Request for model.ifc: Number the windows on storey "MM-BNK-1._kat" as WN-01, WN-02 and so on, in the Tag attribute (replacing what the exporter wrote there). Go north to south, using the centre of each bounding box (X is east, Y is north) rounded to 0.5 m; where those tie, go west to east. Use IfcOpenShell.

First a look at what the model holds.

```python
import ifcopenshell
import ifcopenshell.util.element
import ifcopenshell.util.placement

model = ifcopenshell.open("model.ifc")
print(model.schema)
storey = next(s for s in model.by_type("IfcBuildingStorey") if s.Name == "MM-BNK-1._kat")
windows = [e for e in ifcopenshell.util.element.get_decomposition(storey) if e.is_a("IfcWindow")]
for e in sorted(windows, key=lambda e: e.id()):
    origin = ifcopenshell.util.placement.get_local_placement(e.ObjectPlacement)[:3, 3]
    print(e.id(), e.Tag, e.Name, origin.round(2) + 0.0, sep=" | ")
```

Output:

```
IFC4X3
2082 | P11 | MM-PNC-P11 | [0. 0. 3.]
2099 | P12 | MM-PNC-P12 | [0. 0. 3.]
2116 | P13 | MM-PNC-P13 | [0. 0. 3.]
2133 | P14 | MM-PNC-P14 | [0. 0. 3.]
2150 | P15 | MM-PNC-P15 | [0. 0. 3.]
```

```python
import ifcopenshell
import ifcopenshell.geom
import ifcopenshell.util.element
import ifcopenshell.util.shape

model = ifcopenshell.open("model.ifc")
settings = ifcopenshell.geom.settings()
settings.set("use-world-coords", True)


def centre(element):
    shape = ifcopenshell.geom.create_shape(settings, element)
    return ifcopenshell.util.shape.get_bbox_centroid(shape.geometry)


storey = next(s for s in model.by_type("IfcBuildingStorey") if s.Name == "MM-BNK-1._kat")
windows = [e for e in ifcopenshell.util.element.get_decomposition(storey) if e.is_a("IfcWindow")]

# Insertion points can sit at a corner or the storey origin, so sort by the geometry (in metres).
centres = {e: centre(e) for e in windows}
windows.sort(key=lambda e: (-round(centres[e][1] / 0.5), centres[e][0]))

for i, e in enumerate(windows, start=1):
    number = f"WN-{i:02d}"
    e.Tag = number
    print(e.id(), number)

model.write("model_edited.ifc")
```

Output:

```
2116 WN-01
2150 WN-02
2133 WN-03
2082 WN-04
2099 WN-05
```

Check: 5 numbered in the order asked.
